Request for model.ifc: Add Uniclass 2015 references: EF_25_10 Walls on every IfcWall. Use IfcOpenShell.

First a look at what the model holds.

```python
import ifcopenshell

model = ifcopenshell.open("model.ifc")
print(model.schema)
print("classifications:", [c.Name for c in model.by_type("IfcClassification")])
for ifc_class in ("IfcDoor", "IfcRoof", "IfcStair", "IfcWall", "IfcWindow"):
    print(ifc_class, len(model.by_type(ifc_class)))
```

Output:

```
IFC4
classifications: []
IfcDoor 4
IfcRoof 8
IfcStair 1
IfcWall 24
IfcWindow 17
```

```python
import ifcopenshell
import ifcopenshell.api.classification

model = ifcopenshell.open("model.ifc")

system = ifcopenshell.api.classification.add_classification(model, classification="Uniclass 2015")

codes = {
    "IfcWall": ("EF_25_10", "Walls"),
}
for ifc_class, (code, name) in codes.items():
    products = model.by_type(ifc_class)
    ifcopenshell.api.classification.add_reference(
        model, products=products, classification=system, identification=code, name=name
    )
    print(code, len(products))

model.write("model_edited.ifc")
```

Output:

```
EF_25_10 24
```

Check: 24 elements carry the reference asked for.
